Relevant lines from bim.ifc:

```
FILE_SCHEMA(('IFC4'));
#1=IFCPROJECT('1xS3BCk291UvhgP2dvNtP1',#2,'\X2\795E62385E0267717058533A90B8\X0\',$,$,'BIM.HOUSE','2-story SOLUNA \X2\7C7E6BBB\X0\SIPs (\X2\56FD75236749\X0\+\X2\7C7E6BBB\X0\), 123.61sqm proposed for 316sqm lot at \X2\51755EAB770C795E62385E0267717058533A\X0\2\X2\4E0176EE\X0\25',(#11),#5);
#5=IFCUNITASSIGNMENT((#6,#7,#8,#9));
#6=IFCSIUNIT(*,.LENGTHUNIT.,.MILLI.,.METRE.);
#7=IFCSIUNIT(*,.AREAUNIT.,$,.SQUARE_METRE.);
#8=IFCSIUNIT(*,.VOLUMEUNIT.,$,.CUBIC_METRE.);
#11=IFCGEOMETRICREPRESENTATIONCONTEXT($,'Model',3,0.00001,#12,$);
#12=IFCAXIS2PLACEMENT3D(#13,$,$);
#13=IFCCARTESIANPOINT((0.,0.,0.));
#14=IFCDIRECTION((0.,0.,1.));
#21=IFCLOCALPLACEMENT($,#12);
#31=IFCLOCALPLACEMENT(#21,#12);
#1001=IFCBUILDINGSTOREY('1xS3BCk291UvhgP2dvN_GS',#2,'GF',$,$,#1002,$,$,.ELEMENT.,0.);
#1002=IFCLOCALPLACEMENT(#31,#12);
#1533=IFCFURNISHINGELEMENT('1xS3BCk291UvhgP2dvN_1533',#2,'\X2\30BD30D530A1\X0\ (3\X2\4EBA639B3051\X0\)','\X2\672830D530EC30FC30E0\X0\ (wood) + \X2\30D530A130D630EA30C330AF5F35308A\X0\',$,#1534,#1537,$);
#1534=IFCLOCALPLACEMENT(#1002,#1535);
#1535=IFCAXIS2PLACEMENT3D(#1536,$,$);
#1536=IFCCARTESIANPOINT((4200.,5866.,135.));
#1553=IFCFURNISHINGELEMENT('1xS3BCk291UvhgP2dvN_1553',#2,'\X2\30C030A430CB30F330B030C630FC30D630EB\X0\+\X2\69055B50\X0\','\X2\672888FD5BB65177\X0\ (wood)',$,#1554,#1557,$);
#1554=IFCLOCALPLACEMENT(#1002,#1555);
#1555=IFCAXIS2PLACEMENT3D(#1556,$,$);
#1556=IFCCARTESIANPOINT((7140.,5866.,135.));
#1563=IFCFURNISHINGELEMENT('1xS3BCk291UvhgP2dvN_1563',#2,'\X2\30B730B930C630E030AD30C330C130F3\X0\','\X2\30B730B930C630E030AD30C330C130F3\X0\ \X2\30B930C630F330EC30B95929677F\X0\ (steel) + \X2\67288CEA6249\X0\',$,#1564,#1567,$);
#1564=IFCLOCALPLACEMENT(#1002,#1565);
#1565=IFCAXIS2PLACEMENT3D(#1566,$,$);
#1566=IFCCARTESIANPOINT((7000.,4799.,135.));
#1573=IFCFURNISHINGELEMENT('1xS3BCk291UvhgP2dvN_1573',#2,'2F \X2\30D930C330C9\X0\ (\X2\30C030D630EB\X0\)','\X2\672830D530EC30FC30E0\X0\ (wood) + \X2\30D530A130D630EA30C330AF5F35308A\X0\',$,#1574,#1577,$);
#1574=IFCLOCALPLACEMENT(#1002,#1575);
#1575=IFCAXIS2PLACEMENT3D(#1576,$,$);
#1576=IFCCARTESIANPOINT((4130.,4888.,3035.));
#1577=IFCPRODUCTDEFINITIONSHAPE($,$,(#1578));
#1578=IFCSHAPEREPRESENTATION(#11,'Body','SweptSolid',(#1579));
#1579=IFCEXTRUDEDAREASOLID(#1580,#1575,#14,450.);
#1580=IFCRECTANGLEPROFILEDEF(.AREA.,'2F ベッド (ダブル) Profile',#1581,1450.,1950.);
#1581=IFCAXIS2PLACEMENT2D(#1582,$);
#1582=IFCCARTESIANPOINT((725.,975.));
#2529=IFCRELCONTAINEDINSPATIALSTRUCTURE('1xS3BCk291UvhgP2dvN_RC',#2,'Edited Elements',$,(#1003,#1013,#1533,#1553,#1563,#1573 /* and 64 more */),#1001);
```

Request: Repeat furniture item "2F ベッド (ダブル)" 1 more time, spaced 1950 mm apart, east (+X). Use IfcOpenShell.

```python
import numpy as np
import ifcopenshell
import ifcopenshell.api.geometry
import ifcopenshell.api.root
import ifcopenshell.util.element
import ifcopenshell.util.placement
import ifcopenshell.util.unit

model = ifcopenshell.open("bim.ifc")
unit_scale = ifcopenshell.util.unit.calculate_unit_scale(model)


def reuse_history(source, copy):
    """copy_class also copies each property set's owner history, people and application; keep the originals."""
    for rel in copy.IsDefinedBy:
        if rel.is_a("IfcRelDefinesByProperties") and (history := rel.RelatingPropertyDefinition.OwnerHistory):
            rel.RelatingPropertyDefinition.OwnerHistory = source.OwnerHistory
            ifcopenshell.util.element.remove_deep2(model, history)


source = model.by_guid("1xS3BCk291UvhgP2dvN_1573")
base = ifcopenshell.util.placement.get_local_placement(source.ObjectPlacement)
step = np.array([1.0, 0.0, 0.0]) * 1.95 / unit_scale

for i in range(1, 2):
    copy = ifcopenshell.api.root.copy_class(model, product=source)
    copy.Representation = ifcopenshell.util.element.copy_deep(
        model, source.Representation, exclude=["IfcGeometricRepresentationContext", "IfcRepresentationMap"]
    )
    reuse_history(source, copy)
    matrix = base.copy()
    matrix[:3, 3] += i * step
    print("added at", matrix[:3, 3].round(3) + 0.0)
    ifcopenshell.api.geometry.edit_object_placement(model, product=copy, matrix=matrix, is_si=False)

model.write("bim_v2.ifc")
```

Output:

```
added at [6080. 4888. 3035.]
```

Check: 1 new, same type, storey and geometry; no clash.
